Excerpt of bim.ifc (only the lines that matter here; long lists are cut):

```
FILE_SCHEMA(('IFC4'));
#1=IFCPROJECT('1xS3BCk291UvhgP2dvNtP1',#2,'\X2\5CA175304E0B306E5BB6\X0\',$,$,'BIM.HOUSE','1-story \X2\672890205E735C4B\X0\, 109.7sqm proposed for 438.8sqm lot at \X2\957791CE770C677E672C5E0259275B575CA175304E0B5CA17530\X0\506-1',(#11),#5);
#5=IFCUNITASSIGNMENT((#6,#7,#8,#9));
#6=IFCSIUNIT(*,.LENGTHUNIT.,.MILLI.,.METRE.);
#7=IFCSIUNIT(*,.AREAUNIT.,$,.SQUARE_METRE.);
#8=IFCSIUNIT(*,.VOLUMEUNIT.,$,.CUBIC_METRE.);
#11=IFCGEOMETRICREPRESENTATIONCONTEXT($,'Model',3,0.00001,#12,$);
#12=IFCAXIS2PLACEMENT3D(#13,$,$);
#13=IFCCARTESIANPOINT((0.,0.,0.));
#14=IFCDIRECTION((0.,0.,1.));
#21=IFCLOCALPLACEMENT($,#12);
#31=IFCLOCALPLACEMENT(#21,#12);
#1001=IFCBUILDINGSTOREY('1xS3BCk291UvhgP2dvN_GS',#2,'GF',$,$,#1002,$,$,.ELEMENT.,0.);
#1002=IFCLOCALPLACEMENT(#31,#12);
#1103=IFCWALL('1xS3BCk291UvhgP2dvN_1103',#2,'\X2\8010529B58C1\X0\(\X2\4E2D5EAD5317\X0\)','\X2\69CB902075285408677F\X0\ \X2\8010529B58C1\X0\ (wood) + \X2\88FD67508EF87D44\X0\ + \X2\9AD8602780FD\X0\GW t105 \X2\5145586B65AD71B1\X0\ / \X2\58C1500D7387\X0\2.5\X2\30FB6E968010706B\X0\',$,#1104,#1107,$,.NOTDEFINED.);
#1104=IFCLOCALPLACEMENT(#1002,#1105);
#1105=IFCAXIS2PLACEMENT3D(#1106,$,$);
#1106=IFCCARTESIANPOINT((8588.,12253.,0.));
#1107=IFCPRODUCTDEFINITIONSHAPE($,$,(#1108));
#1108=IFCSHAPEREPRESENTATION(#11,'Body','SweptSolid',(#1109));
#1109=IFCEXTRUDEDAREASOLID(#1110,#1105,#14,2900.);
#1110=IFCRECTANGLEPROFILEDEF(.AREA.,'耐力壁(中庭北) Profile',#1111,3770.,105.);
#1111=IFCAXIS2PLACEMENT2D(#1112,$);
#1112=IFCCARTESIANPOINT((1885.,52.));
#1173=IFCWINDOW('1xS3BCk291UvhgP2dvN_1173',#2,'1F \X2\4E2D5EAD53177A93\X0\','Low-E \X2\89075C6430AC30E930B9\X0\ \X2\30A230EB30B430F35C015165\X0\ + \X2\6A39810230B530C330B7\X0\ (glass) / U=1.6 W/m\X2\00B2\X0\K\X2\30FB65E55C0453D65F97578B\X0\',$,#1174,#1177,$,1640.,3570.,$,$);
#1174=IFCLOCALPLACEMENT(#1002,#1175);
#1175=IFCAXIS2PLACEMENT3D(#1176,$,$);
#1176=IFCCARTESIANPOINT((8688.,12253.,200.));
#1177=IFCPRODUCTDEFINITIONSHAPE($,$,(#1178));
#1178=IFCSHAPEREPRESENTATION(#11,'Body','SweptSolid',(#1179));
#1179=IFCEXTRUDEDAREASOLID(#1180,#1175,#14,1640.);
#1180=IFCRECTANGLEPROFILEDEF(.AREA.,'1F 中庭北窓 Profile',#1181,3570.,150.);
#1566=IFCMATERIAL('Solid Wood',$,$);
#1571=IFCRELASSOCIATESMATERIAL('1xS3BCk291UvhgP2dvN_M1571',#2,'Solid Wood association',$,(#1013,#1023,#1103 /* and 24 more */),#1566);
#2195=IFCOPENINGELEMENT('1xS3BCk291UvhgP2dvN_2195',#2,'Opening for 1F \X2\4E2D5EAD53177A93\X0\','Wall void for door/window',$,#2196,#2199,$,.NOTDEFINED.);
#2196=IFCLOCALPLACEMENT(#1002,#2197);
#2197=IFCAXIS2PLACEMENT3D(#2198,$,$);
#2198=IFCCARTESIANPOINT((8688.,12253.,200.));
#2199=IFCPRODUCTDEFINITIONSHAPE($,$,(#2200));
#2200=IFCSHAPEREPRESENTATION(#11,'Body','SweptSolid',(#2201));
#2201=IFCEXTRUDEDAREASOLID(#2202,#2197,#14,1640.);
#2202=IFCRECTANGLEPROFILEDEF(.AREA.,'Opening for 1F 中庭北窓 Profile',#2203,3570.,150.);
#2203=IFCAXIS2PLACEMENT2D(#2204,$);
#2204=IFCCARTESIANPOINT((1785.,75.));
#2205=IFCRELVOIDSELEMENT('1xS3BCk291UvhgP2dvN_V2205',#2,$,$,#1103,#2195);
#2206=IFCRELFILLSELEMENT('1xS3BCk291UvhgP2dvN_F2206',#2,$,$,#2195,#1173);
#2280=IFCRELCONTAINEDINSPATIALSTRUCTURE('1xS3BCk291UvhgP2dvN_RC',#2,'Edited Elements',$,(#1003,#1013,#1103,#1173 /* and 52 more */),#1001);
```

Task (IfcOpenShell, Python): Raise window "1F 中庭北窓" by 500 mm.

```python
import numpy as np
import ifcopenshell
import ifcopenshell.api.geometry
import ifcopenshell.util.placement
import ifcopenshell.util.unit

model = ifcopenshell.open("bim.ifc")
unit_scale = ifcopenshell.util.unit.calculate_unit_scale(model)

window = model.by_id(1173)
opening = window.FillsVoids[0].RelatingOpeningElement
dz = 0.5 / unit_scale

shift = np.array([0.0, 0.0, dz])
# The window is not placed relative to its opening, so move both.
for product in (opening, window):
    matrix = ifcopenshell.util.placement.get_local_placement(product.ObjectPlacement)
    matrix[:3, 3] += shift
    ifcopenshell.api.geometry.edit_object_placement(model, product=product, matrix=matrix, is_si=False)

print(f"moved by {dz * unit_scale:+.3f} m")

model.write("bim-out.ifc")
```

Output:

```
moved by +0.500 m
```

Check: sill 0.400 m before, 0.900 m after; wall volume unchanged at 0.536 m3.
